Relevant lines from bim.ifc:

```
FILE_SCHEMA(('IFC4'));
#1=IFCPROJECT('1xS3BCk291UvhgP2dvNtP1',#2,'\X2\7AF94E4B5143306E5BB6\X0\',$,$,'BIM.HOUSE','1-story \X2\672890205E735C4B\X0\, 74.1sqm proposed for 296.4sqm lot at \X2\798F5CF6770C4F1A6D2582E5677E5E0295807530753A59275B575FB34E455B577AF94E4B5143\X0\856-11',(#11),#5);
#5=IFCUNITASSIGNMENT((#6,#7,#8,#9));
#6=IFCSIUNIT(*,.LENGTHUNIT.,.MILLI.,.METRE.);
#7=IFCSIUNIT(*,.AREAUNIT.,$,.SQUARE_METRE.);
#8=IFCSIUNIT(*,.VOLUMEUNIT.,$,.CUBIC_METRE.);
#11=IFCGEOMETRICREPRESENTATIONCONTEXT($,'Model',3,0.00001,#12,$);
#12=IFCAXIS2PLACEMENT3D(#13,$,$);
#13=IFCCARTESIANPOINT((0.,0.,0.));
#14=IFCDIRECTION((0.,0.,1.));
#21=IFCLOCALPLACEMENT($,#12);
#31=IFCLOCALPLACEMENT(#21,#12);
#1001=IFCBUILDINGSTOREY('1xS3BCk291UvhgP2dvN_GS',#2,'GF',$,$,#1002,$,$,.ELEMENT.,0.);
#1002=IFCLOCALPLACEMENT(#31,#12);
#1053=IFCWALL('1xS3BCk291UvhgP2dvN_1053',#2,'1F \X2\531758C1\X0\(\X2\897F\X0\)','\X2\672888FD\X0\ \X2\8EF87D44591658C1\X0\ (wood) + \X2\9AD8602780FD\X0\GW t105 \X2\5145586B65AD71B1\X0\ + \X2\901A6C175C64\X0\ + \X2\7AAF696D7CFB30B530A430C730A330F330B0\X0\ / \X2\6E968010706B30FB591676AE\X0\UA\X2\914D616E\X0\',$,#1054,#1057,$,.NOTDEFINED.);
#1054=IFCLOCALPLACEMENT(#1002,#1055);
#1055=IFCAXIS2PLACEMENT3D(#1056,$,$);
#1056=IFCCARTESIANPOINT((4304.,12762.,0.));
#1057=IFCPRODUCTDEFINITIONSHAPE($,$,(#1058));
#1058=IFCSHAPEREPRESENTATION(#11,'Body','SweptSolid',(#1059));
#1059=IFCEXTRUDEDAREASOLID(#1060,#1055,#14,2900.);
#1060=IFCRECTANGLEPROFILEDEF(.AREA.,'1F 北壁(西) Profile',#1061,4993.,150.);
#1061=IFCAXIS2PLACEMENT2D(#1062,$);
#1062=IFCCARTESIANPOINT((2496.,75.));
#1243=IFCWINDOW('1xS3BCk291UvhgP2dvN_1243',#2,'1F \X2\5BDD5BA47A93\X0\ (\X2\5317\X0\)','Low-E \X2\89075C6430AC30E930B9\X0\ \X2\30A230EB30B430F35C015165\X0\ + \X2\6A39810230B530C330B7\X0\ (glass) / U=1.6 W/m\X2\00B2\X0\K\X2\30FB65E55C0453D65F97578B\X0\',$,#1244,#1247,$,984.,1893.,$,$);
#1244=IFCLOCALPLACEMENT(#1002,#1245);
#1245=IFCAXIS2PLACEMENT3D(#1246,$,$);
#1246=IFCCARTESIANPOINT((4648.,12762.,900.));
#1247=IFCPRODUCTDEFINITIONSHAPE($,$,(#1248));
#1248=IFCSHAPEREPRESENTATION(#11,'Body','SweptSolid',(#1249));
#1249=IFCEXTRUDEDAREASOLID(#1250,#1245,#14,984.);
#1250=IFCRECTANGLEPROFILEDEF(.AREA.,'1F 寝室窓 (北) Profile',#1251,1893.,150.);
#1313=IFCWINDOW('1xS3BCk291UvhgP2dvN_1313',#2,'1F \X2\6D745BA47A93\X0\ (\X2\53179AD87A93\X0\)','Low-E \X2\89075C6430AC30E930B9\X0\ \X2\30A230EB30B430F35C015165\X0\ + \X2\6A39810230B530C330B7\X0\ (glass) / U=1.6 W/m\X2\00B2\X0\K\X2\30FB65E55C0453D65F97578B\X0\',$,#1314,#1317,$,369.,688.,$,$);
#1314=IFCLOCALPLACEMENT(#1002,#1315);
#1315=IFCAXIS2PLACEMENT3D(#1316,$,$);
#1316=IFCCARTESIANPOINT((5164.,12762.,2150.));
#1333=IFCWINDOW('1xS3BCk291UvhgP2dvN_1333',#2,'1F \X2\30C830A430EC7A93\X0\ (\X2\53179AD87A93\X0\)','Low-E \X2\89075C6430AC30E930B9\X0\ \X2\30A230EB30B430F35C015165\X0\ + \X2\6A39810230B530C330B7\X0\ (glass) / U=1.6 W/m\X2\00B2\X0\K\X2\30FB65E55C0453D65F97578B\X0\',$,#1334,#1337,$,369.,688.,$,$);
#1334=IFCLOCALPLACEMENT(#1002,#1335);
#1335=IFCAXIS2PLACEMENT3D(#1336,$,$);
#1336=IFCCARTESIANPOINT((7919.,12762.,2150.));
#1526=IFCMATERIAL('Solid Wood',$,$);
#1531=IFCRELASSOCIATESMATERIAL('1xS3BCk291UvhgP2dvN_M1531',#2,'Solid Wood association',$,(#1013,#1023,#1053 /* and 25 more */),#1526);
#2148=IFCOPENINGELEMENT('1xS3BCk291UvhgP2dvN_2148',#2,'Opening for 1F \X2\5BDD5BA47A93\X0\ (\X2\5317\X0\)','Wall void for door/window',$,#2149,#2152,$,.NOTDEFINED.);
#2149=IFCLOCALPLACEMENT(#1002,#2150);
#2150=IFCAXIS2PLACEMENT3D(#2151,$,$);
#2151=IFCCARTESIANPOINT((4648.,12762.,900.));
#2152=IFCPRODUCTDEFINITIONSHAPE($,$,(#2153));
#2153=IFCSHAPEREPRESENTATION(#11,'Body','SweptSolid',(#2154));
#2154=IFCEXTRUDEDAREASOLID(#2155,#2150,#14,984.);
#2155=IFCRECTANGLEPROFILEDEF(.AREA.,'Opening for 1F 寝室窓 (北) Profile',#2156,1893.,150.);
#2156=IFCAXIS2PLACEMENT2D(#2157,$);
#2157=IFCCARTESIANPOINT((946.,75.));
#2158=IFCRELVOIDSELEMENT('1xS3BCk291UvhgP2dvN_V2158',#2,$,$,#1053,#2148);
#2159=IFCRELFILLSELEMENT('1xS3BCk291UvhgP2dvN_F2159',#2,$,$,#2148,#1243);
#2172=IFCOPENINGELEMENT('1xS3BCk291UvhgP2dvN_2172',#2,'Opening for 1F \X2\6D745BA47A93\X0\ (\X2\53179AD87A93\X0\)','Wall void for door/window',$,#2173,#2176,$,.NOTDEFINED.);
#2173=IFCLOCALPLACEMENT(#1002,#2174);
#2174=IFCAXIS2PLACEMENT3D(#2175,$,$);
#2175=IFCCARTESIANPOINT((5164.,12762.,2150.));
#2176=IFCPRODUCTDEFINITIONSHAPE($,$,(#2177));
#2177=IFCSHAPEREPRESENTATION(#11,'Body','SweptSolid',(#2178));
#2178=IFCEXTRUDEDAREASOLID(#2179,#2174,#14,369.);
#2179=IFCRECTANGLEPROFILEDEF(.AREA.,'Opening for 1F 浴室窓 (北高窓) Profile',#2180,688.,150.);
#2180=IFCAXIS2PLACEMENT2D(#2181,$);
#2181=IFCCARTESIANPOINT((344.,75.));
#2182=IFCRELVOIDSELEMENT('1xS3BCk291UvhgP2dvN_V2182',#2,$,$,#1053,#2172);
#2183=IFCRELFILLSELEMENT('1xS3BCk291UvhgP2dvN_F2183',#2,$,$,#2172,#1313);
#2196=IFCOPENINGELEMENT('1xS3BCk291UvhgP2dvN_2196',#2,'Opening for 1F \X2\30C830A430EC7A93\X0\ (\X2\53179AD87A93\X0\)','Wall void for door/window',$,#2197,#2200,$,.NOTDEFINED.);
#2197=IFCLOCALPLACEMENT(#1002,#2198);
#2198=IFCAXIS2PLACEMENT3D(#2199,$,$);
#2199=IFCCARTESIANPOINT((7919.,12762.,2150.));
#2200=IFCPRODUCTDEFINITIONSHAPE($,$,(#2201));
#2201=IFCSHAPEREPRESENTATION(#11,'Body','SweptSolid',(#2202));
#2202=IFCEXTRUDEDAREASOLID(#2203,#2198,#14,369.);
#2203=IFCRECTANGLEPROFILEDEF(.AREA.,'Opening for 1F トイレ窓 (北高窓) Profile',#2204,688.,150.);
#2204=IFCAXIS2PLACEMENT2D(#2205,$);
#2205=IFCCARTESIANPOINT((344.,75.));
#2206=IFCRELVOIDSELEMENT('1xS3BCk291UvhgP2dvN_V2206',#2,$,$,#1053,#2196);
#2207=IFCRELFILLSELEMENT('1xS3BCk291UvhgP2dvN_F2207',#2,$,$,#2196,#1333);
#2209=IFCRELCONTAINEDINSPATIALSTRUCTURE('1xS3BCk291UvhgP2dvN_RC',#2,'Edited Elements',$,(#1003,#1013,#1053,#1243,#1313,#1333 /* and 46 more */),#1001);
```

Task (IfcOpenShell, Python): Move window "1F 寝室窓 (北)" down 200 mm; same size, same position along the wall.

```python
import numpy as np
import ifcopenshell
import ifcopenshell.api.geometry
import ifcopenshell.util.placement
import ifcopenshell.util.unit

model = ifcopenshell.open("bim.ifc")
unit_scale = ifcopenshell.util.unit.calculate_unit_scale(model)

window = model.by_guid("1xS3BCk291UvhgP2dvN_1243")
opening = window.FillsVoids[0].RelatingOpeningElement
dz = -0.2 / unit_scale

shift = np.array([0.0, 0.0, dz])
# The window is not placed relative to its opening, so move both.
for product in (opening, window):
    matrix = ifcopenshell.util.placement.get_local_placement(product.ObjectPlacement)
    matrix[:3, 3] += shift
    ifcopenshell.api.geometry.edit_object_placement(model, product=product, matrix=matrix, is_si=False)

print(f"moved by {dz * unit_scale:+.3f} m")

model.write("bim_v2.ifc")
```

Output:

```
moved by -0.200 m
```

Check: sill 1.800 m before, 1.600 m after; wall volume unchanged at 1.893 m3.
